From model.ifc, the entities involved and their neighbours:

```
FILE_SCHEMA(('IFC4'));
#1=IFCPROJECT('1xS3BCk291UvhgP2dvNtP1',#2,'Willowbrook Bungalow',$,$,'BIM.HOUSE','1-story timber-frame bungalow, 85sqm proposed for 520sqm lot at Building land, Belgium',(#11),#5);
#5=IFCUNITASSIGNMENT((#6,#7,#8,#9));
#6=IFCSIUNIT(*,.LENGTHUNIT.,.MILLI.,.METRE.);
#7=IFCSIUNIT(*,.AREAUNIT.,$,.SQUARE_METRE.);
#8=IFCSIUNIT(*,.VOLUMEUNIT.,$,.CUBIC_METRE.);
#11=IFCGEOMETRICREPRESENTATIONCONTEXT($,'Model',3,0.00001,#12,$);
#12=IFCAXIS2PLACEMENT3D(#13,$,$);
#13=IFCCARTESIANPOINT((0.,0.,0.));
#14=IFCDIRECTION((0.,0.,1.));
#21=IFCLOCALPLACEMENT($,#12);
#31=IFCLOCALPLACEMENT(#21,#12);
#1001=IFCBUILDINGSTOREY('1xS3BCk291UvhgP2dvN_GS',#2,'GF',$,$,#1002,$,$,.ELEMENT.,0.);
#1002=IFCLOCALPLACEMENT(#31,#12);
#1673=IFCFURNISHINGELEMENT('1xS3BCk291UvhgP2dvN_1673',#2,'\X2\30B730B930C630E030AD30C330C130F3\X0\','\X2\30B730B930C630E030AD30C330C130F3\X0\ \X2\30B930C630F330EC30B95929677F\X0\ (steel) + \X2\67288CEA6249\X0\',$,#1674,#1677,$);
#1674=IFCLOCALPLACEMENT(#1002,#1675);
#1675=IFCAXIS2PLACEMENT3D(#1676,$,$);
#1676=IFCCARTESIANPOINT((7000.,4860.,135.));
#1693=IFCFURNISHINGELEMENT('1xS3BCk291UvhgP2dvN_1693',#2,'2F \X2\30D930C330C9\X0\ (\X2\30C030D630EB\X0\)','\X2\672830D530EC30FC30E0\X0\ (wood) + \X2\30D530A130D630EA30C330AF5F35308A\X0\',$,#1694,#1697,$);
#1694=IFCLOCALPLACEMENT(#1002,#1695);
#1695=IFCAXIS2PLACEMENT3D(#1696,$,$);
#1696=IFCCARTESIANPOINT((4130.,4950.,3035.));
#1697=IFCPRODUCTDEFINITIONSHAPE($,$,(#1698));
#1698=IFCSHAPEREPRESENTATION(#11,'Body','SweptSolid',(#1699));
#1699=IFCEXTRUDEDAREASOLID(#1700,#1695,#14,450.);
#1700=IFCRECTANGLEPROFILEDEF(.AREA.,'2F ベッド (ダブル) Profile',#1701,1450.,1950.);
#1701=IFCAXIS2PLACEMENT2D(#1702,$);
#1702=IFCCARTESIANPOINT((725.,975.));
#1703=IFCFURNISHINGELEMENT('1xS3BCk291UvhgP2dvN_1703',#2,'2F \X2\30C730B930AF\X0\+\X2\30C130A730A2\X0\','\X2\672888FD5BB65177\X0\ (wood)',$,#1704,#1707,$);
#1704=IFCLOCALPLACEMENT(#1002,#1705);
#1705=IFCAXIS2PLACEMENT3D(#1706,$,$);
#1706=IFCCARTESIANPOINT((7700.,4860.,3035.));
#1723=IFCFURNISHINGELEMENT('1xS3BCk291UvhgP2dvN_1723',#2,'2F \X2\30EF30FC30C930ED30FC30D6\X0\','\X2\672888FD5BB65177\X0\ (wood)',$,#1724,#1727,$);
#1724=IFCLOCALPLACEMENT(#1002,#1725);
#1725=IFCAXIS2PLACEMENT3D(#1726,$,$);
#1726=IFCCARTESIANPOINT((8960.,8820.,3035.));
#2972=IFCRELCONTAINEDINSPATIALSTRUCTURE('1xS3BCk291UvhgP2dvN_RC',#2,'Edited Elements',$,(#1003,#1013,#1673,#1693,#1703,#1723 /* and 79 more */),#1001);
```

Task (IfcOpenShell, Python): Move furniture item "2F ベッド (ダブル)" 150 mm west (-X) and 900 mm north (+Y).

```python
import ifcopenshell
import ifcopenshell.api.geometry
import ifcopenshell.util.placement

model = ifcopenshell.open("model.ifc")

item = model.by_id(1693)
matrix = ifcopenshell.util.placement.get_local_placement(item.ObjectPlacement)
matrix[0, 3] -= 150.0
matrix[1, 3] += 900.0
ifcopenshell.api.geometry.edit_object_placement(model, product=item, matrix=matrix, is_si=False)

print(ifcopenshell.util.placement.get_local_placement(item.ObjectPlacement).round(3) + 0.0)

model.write("model_rev.ifc")
```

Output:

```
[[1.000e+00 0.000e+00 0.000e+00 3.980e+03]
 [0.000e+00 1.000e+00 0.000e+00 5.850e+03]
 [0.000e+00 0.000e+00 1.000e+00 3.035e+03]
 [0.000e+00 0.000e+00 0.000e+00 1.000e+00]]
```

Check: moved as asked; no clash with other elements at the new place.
